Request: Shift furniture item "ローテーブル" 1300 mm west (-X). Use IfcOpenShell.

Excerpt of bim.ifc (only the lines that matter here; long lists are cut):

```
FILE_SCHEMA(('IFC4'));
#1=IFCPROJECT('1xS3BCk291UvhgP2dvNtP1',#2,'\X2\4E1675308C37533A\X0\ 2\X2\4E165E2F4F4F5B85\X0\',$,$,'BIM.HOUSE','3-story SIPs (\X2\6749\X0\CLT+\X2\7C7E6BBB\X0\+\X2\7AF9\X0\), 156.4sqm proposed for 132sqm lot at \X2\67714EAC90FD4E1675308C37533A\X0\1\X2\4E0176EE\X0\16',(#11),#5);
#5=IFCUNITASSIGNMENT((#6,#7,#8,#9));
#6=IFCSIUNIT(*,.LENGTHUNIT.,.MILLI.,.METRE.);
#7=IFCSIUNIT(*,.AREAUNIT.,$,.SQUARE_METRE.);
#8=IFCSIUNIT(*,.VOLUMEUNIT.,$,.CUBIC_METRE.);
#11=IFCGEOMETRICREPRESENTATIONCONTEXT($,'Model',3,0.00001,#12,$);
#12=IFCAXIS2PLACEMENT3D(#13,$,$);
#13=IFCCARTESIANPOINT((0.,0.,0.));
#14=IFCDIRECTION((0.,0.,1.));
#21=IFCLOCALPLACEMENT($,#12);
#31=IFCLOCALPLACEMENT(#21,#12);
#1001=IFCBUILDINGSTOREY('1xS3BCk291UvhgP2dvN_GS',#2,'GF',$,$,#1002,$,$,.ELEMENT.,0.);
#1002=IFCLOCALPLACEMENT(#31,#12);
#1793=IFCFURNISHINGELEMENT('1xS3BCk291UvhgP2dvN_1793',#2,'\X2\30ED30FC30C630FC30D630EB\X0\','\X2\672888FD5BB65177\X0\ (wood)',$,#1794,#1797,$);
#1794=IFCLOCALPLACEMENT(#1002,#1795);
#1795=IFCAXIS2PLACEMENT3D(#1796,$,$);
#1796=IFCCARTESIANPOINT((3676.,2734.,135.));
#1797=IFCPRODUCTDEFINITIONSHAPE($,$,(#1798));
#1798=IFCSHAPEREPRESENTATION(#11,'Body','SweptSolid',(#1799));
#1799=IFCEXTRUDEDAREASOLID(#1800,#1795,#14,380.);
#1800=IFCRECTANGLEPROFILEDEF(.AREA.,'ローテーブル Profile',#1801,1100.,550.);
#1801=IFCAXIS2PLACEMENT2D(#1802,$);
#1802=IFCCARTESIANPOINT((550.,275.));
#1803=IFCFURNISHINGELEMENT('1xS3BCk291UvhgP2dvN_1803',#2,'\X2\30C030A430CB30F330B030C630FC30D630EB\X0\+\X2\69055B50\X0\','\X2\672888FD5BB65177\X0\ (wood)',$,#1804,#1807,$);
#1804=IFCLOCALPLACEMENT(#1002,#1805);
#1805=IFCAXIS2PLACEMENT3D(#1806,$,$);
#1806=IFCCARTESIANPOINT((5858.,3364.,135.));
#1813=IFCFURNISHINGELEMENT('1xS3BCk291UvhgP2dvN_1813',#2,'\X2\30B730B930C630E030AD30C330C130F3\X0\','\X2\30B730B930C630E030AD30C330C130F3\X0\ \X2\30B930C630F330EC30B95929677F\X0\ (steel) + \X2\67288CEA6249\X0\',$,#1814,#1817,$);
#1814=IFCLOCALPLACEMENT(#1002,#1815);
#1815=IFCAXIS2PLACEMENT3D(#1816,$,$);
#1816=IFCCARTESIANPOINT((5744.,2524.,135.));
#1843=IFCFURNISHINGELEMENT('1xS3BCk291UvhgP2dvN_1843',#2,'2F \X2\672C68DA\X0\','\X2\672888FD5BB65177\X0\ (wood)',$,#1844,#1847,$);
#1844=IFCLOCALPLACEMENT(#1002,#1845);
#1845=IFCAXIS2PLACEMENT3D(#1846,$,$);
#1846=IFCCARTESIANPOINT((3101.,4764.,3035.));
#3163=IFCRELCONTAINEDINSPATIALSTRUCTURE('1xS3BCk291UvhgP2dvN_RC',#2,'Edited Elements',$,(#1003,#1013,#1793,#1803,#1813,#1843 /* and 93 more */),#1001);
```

```python
import ifcopenshell
import ifcopenshell.api.geometry
import ifcopenshell.util.placement
import ifcopenshell.util.unit

model = ifcopenshell.open("bim.ifc")
unit_scale = ifcopenshell.util.unit.calculate_unit_scale(model)

item = model.by_id(1793)
matrix = ifcopenshell.util.placement.get_local_placement(item.ObjectPlacement)
matrix[0, 3] -= 1.3 / unit_scale
ifcopenshell.api.geometry.edit_object_placement(model, product=item, matrix=matrix, is_si=False)

print(ifcopenshell.util.placement.get_local_placement(item.ObjectPlacement).round(3) + 0.0)

model.write("bim_rev.ifc")
```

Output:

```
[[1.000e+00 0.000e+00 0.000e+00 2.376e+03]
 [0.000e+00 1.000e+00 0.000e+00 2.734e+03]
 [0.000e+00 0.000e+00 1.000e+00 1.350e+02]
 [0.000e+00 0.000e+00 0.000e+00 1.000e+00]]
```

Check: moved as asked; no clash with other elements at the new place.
